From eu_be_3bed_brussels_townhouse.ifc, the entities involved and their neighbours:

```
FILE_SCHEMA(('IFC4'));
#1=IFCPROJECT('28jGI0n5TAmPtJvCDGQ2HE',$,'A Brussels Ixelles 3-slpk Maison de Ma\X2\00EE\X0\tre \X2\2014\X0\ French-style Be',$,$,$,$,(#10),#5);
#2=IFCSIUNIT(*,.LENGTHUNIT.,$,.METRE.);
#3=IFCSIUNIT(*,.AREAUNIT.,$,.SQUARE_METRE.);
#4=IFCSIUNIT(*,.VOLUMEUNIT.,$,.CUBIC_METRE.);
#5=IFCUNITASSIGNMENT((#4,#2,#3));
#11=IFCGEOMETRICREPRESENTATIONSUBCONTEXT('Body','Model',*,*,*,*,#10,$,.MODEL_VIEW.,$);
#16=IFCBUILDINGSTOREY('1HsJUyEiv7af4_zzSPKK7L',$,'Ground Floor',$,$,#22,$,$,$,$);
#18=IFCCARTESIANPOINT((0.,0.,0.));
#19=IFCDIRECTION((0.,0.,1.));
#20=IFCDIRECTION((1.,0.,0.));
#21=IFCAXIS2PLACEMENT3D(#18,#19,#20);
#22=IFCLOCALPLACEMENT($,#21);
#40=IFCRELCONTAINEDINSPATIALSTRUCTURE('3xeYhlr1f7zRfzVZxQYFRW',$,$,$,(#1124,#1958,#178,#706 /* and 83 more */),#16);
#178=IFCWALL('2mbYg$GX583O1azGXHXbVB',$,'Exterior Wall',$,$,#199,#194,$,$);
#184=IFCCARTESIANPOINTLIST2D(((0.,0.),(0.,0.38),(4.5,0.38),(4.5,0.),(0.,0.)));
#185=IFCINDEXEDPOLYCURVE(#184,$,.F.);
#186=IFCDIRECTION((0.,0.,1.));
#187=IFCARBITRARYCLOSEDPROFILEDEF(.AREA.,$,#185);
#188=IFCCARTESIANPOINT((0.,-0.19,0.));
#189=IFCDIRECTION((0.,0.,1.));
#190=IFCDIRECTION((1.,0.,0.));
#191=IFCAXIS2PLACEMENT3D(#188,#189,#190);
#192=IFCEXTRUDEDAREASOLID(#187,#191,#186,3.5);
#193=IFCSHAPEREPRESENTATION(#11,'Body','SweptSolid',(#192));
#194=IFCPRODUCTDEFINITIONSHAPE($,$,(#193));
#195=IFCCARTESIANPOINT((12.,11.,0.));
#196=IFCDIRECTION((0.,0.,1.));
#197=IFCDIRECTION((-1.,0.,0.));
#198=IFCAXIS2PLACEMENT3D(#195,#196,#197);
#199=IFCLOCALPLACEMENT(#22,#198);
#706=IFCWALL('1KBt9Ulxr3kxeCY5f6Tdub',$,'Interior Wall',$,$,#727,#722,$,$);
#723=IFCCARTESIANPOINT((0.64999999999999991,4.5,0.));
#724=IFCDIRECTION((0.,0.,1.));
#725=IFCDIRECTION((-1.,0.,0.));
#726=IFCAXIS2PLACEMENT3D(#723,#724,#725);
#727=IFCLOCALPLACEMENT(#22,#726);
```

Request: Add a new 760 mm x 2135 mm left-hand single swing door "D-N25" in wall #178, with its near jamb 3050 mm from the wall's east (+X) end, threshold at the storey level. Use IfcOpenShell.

```python
import numpy as np
import ifcopenshell
import ifcopenshell.api.feature
import ifcopenshell.api.geometry
import ifcopenshell.api.root
import ifcopenshell.api.spatial
import ifcopenshell.geom
import ifcopenshell.util.element
import ifcopenshell.util.placement
import ifcopenshell.util.representation
import ifcopenshell.util.shape
import ifcopenshell.util.unit

model = ifcopenshell.open("eu_be_3bed_brussels_townhouse.ifc")
unit_scale = ifcopenshell.util.unit.calculate_unit_scale(model)
settings = ifcopenshell.geom.settings()


def volume(element):
    """Net volume in cubic metres, openings subtracted."""
    shape = ifcopenshell.geom.create_shape(settings, element)
    return ifcopenshell.util.shape.get_volume(shape.geometry)


wall = model.by_guid("2mbYg$GX583O1azGXHXbVB")
storey = ifcopenshell.util.element.get_container(wall, ifc_class="IfcBuildingStorey")
context = ifcopenshell.util.representation.get_context(model, "Model", "Body", "MODEL_VIEW")
before = volume(wall)

width, height, from_end, sill = 0.76, 2.135, 3.05, 0.0  # metres

# The wall runs along its own X axis, and the end named is its -X end.
wall_shape = ifcopenshell.geom.create_shape(settings, wall)
x, y, z = ifcopenshell.util.shape.get_vertices(wall_shape.geometry).T
start = x.min() + from_end
face, thickness = float(y.min()), float(y.max() - y.min())
wall_matrix = ifcopenshell.util.placement.get_local_placement(wall.ObjectPlacement)
level = ifcopenshell.util.placement.get_local_placement(storey.ObjectPlacement)[2, 3]


def in_wall(x, y):
    """Placement at x, y metres in the wall's axes, at sill height."""
    matrix = wall_matrix.copy()
    matrix[:, 3] = wall_matrix @ np.array([x / unit_scale, y / unit_scale, 0.0, 1.0])
    matrix[2, 3] = level + sill / unit_scale
    return matrix


# Opening: a box that overshoots both wall faces by 50 mm.
opening = ifcopenshell.api.root.create_entity(model, ifc_class="IfcOpeningElement", predefined_type="OPENING")
box = ifcopenshell.api.geometry.add_wall_representation(
    model, context=context, length=width, height=height, thickness=thickness + 0.1
)
ifcopenshell.api.geometry.assign_representation(model, product=opening, representation=box)
ifcopenshell.api.geometry.edit_object_placement(model, product=opening, matrix=in_wall(start, face - 0.05), is_si=False)
ifcopenshell.api.feature.add_feature(model, feature=opening, element=wall)

door = ifcopenshell.api.root.create_entity(model, ifc_class="IfcDoor", name="D-N25", predefined_type="DOOR")
door.OverallWidth, door.OverallHeight = width / unit_scale, height / unit_scale
door.OperationType = "SINGLE_SWING_LEFT"
body = ifcopenshell.api.geometry.add_door_representation(
    model,
    context=context,
    overall_width=door.OverallWidth,
    overall_height=door.OverallHeight,
    operation_type="SINGLE_SWING_LEFT",
    lining_properties={"LiningDepth": thickness / unit_scale, "ThresholdDepth": thickness / unit_scale},
)
ifcopenshell.api.geometry.assign_representation(model, product=door, representation=body)
ifcopenshell.api.spatial.assign_container(model, products=[door], relating_structure=storey)
ifcopenshell.api.feature.add_filling(model, opening=opening, element=door)

# The lining spans the wall, so the door starts at the wall face.
ifcopenshell.api.geometry.edit_object_placement(model, product=door, matrix=in_wall(start, face), is_si=False)

after = volume(wall)

print(f"wall volume {before:.3f} -> {after:.3f} m3")

model.write("eu_be_3bed_brussels_townhouse-out.ifc")
```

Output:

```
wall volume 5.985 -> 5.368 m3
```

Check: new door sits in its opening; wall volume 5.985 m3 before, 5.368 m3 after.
